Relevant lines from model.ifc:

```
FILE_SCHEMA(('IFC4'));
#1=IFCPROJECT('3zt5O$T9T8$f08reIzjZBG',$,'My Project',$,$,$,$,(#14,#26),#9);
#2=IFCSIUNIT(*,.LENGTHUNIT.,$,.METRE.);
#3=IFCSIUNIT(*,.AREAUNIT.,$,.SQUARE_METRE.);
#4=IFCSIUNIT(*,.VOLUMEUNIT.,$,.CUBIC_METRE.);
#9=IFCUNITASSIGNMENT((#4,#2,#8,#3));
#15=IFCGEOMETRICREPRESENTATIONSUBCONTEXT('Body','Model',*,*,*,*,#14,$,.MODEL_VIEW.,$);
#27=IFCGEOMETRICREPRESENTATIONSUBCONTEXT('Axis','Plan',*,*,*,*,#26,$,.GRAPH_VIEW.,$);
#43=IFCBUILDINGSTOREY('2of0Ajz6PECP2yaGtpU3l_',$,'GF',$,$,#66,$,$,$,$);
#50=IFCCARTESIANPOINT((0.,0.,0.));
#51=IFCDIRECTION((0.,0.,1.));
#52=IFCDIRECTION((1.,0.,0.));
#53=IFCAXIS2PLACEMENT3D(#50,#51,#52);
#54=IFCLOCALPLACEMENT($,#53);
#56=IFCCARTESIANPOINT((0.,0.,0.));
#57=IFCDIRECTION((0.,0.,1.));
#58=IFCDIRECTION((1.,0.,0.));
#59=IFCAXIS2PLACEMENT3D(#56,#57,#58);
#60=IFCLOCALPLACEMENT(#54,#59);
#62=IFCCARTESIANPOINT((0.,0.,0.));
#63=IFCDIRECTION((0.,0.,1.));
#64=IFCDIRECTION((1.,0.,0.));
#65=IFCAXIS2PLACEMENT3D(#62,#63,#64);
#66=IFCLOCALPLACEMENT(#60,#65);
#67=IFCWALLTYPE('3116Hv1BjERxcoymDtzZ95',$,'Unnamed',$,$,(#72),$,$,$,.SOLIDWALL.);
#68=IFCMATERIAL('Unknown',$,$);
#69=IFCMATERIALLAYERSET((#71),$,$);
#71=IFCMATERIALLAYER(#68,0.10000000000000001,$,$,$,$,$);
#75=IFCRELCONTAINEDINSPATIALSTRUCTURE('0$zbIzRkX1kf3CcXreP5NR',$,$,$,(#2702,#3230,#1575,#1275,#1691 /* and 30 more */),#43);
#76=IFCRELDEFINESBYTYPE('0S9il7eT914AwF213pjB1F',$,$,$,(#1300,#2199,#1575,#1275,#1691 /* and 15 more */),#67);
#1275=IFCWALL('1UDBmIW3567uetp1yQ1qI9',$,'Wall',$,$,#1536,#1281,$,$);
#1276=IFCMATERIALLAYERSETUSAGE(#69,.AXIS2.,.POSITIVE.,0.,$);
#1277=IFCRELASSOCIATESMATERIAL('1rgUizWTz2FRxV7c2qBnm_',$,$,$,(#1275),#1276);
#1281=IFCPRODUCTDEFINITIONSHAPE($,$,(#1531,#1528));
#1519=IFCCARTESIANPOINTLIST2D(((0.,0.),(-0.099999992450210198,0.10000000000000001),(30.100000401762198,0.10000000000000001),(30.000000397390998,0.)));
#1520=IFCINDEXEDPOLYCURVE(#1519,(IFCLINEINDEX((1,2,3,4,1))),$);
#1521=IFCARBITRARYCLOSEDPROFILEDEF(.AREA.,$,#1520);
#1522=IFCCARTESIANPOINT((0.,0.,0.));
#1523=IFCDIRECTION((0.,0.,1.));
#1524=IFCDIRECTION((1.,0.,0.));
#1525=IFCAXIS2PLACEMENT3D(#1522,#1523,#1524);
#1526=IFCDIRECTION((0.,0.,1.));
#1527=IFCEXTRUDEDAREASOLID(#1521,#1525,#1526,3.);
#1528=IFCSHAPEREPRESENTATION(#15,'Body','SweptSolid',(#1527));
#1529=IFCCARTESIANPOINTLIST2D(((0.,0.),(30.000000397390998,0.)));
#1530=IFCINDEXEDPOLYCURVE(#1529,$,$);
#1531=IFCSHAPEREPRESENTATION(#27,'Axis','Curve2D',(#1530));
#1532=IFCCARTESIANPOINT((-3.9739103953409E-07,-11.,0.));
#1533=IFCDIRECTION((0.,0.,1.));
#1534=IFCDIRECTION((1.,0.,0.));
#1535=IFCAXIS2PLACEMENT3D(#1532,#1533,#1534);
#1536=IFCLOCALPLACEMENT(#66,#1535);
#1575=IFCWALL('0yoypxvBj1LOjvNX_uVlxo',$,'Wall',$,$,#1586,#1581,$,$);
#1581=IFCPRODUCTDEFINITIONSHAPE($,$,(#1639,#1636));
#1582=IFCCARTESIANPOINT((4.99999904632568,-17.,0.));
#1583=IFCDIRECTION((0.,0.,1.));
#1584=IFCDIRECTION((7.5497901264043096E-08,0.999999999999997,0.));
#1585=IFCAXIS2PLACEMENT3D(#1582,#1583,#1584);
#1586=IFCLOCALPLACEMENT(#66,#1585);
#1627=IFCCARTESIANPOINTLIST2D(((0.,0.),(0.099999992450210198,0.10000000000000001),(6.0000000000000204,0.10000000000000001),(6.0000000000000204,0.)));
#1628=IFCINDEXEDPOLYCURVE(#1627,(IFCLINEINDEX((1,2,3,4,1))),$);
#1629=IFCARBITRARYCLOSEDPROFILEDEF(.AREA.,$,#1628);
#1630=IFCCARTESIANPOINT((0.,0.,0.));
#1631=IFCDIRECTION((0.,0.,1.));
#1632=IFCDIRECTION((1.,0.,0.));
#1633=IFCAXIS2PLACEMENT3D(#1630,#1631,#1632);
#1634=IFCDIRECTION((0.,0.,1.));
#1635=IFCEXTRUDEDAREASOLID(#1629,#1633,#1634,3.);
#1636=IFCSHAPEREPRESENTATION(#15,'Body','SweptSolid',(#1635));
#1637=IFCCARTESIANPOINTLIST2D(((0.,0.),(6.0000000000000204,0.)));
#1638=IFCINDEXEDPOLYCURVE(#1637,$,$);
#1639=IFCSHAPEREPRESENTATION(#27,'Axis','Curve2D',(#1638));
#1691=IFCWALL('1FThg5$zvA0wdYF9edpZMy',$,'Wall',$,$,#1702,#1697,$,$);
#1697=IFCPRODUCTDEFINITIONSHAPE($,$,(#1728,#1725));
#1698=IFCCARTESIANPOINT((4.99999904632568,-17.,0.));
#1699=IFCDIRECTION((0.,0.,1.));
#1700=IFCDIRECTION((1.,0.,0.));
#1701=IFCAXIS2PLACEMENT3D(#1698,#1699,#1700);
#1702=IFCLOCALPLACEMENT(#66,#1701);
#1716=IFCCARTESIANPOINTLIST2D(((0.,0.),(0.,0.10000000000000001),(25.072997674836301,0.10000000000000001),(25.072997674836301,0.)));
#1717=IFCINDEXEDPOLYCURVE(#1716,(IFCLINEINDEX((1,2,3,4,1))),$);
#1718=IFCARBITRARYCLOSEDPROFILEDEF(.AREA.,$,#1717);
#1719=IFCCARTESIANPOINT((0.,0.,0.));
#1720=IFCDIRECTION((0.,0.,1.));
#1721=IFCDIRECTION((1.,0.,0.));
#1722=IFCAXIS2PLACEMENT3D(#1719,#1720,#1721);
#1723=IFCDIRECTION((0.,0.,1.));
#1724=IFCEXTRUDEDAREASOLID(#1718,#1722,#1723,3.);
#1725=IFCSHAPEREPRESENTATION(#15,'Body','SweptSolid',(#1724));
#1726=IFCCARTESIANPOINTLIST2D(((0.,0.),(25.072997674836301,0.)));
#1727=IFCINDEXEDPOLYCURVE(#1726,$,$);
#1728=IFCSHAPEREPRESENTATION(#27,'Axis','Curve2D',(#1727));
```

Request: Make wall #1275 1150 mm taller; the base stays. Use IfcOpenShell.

```python
import ifcopenshell
import ifcopenshell.geom
import ifcopenshell.util.representation
import ifcopenshell.util.shape
import ifcopenshell.util.unit

model = ifcopenshell.open("model.ifc")
unit_scale = ifcopenshell.util.unit.calculate_unit_scale(model)
settings = ifcopenshell.geom.settings()


def volume(element):
    """Net volume in cubic metres, openings subtracted."""
    shape = ifcopenshell.geom.create_shape(settings, element)
    return ifcopenshell.util.shape.get_volume(shape.geometry)


wall = model.by_id(1275)
before = volume(wall)

body = ifcopenshell.util.representation.get_representation(wall, "Model", "Body")
solid = body.Items[0]
old_height = solid.Depth
solid.Depth += 1.15 / unit_scale
after = volume(wall)

print(f"height {old_height:g} -> {solid.Depth:g}, volume {before:.3f} -> {after:.3f} m3")

model.write("model_v2.ifc")
```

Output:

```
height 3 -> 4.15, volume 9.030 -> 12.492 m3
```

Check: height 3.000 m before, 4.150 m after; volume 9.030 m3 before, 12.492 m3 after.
